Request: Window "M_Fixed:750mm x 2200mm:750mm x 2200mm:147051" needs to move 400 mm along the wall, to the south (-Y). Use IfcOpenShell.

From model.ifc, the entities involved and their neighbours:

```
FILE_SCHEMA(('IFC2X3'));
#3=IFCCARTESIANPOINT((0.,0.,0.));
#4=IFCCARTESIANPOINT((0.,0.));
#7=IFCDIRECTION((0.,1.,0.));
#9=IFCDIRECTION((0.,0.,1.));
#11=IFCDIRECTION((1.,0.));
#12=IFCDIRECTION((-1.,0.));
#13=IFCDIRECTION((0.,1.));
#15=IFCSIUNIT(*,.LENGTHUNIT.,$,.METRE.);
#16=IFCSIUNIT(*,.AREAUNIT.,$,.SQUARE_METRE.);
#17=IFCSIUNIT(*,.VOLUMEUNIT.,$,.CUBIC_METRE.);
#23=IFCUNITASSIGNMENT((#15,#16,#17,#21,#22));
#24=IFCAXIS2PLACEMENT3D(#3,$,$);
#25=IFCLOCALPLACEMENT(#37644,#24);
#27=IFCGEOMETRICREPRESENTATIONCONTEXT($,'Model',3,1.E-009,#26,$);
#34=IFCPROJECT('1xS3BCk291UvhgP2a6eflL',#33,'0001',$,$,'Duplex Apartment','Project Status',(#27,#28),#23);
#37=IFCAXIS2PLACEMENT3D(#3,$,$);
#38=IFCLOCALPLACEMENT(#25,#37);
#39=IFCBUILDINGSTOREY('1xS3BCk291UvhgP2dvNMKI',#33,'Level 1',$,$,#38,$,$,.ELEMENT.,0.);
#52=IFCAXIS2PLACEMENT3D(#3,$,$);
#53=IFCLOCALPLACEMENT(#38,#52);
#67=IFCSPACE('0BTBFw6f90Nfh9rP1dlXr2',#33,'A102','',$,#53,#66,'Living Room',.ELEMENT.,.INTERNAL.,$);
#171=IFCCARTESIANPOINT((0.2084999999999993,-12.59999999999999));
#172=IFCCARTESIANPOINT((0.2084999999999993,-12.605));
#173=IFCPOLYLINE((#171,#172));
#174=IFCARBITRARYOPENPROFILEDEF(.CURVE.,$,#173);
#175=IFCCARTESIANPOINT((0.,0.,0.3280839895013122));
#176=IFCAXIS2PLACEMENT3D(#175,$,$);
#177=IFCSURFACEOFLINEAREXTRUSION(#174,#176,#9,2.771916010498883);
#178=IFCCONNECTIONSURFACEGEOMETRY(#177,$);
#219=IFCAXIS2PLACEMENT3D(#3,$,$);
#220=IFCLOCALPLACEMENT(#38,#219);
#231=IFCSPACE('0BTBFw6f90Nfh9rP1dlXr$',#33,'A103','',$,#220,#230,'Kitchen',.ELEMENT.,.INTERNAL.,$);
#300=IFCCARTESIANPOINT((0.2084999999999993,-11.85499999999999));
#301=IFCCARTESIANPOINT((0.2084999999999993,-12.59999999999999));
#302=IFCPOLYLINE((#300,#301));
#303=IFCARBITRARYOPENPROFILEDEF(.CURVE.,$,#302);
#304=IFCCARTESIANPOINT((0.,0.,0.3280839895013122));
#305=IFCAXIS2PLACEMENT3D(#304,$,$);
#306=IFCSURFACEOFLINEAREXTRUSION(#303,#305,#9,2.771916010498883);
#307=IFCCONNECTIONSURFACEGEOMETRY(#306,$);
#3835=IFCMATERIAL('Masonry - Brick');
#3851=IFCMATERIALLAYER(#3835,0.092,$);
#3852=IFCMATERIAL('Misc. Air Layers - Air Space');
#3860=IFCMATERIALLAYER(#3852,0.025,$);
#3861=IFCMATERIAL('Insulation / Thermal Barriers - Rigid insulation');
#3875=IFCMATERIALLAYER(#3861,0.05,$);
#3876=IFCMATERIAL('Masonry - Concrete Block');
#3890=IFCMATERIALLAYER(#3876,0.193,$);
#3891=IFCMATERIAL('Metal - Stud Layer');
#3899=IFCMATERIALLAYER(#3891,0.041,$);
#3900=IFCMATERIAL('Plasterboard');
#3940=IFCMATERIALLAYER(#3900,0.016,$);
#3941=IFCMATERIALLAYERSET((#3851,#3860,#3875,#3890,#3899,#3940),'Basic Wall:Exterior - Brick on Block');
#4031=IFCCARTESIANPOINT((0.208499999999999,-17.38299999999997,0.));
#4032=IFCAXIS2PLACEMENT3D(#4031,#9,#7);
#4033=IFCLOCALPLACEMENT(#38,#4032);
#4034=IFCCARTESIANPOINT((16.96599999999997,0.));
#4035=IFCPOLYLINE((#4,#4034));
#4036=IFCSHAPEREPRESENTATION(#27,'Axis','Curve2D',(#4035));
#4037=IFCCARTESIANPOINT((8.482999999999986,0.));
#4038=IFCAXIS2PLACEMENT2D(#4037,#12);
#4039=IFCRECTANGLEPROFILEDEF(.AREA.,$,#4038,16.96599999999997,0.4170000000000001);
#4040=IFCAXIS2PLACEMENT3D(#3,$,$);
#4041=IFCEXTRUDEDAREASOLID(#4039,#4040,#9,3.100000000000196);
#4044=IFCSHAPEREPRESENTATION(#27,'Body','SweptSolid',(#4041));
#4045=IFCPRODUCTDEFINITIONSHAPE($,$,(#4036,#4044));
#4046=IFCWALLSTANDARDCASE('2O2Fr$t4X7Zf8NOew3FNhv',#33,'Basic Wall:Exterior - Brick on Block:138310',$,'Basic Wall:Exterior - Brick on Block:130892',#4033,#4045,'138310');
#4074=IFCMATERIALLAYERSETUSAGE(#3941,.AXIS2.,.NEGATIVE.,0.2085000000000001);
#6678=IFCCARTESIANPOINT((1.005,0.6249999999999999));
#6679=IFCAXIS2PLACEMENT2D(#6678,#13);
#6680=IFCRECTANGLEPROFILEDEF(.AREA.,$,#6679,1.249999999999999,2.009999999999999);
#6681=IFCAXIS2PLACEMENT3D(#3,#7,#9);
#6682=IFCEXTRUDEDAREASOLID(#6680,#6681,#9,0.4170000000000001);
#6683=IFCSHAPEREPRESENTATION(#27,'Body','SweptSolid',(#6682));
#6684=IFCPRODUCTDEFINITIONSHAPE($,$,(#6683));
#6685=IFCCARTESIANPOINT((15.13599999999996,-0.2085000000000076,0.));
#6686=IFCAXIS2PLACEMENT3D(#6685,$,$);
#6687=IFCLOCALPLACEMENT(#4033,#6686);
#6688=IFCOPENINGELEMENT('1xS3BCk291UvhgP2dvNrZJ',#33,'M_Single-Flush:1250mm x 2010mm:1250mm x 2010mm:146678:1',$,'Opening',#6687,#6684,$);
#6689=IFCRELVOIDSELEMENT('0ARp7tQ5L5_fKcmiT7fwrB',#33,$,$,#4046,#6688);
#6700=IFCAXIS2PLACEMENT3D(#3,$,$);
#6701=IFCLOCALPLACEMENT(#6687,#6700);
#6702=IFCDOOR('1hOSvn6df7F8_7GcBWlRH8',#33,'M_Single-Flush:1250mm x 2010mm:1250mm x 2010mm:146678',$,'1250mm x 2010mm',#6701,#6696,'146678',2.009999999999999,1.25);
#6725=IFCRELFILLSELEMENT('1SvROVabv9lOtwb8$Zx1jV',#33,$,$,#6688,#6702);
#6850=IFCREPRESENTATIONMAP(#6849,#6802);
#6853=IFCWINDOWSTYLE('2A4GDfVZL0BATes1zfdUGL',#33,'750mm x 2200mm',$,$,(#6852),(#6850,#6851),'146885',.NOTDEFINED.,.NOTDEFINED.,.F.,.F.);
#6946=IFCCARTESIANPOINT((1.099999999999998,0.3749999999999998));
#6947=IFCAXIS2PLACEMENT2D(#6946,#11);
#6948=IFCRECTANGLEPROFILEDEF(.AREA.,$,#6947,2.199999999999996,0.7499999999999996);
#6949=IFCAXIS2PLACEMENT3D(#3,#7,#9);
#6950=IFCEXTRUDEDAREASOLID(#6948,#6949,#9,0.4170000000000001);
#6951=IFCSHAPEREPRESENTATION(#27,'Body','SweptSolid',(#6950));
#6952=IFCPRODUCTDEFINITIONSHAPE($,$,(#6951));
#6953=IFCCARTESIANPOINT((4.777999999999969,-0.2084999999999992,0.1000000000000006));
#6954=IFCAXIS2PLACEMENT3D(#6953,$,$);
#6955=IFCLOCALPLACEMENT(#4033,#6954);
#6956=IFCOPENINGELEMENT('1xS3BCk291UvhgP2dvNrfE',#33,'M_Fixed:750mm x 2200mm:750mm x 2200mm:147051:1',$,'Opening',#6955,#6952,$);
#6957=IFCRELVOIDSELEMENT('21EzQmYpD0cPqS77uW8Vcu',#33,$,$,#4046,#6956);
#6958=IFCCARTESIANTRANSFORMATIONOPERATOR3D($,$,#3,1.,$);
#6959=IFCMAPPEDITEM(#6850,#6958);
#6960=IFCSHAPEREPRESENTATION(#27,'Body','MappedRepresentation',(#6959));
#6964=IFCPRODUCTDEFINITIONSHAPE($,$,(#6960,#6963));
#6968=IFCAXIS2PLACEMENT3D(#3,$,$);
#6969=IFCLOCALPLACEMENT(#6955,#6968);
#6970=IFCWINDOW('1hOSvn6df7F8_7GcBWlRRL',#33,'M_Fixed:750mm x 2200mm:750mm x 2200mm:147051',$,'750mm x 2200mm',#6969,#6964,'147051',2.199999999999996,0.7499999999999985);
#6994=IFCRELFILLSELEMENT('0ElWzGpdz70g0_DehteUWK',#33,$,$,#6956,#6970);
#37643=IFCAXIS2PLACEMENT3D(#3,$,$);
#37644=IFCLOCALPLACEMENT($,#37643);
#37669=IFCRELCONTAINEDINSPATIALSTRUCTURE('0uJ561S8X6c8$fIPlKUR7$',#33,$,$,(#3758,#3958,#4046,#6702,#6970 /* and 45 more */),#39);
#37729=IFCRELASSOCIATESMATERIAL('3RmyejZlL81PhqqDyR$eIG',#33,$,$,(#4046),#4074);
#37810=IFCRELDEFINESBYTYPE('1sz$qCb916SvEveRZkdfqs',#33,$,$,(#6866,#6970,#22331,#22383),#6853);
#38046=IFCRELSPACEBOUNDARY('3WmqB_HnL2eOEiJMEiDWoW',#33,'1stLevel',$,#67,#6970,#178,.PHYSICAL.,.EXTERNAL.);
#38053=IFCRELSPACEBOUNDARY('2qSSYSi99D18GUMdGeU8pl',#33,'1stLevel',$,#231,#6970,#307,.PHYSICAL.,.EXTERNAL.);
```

```python
import numpy as np
import ifcopenshell
import ifcopenshell.api.geometry
import ifcopenshell.util.placement
import ifcopenshell.util.unit

model = ifcopenshell.open("model.ifc")
unit_scale = ifcopenshell.util.unit.calculate_unit_scale(model)

window = model.by_id(6970)
opening = window.FillsVoids[0].RelatingOpeningElement
wall = opening.VoidsElements[0].RelatingBuildingElement

wall_matrix = ifcopenshell.util.placement.get_local_placement(wall.ObjectPlacement)
shift = wall_matrix[:3, 0] * -0.4 / unit_scale
before = ifcopenshell.util.placement.get_local_placement(window.ObjectPlacement)[:3, 3].copy()

# The window is placed relative to its opening, so it follows when the opening moves.
matrix = ifcopenshell.util.placement.get_local_placement(opening.ObjectPlacement)
matrix[:3, 3] += shift
ifcopenshell.api.geometry.edit_object_placement(
    model, product=opening, matrix=matrix, is_si=False, should_transform_children=True
)

# Space boundary surfaces are stored in each space's coordinates; move them too.
for rel in window.ProvidesBoundaries:
    if not rel.ConnectionGeometry:
        continue
    surface = rel.ConnectionGeometry.SurfaceOnRelatingElement
    space_matrix = ifcopenshell.util.placement.get_local_placement(rel.RelatingSpace.ObjectPlacement)
    point = np.array(surface.Position.Location.Coordinates) + space_matrix[:3, :3].T @ shift
    surface.Position = model.createIfcAxis2Placement3D(
        model.createIfcCartesianPoint(point.tolist()), surface.Position.Axis, surface.Position.RefDirection
    )

after = ifcopenshell.util.placement.get_local_placement(window.ObjectPlacement)[:3, 3]
print("window moved by", (after - before).round(3) + 0.0)

model.write("model_v2.ifc")
```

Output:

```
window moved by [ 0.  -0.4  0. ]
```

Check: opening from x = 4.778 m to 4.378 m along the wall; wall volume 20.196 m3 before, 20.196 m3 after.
